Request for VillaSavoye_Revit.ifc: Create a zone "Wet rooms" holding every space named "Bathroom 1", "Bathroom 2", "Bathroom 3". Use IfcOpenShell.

First a look at what the model holds.

```python
import ifcopenshell

model = ifcopenshell.open("VillaSavoye_Revit.ifc")
print(model.schema)
seen = {}
for space in model.by_type("IfcSpace"):
    seen[space.LongName] = seen.get(space.LongName, 0) + 1
for name, count in sorted(seen.items(), key=str):
    print(count, "x", name)
print("zones:", [z.Name for z in model.by_type("IfcZone")][:20])
```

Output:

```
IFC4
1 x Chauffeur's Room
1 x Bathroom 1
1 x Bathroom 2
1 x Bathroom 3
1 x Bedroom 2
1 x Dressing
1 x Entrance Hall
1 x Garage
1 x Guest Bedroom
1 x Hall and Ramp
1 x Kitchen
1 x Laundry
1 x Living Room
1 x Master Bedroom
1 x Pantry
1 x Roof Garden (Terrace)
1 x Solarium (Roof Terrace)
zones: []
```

```python
import ifcopenshell
import ifcopenshell.api.group
import ifcopenshell.api.root

model = ifcopenshell.open("VillaSavoye_Revit.ifc")

names = {"Bathroom 1", "Bathroom 2", "Bathroom 3"}
spaces = [s for s in model.by_type("IfcSpace") if s.LongName in names]

zone = ifcopenshell.api.root.create_entity(model, ifc_class="IfcZone", name="Wet rooms")
ifcopenshell.api.group.assign_group(model, products=spaces, group=zone)
print(len(spaces), "spaces in", zone.Name)

model.write("VillaSavoye_Revit-out.ifc")
```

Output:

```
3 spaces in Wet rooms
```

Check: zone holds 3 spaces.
